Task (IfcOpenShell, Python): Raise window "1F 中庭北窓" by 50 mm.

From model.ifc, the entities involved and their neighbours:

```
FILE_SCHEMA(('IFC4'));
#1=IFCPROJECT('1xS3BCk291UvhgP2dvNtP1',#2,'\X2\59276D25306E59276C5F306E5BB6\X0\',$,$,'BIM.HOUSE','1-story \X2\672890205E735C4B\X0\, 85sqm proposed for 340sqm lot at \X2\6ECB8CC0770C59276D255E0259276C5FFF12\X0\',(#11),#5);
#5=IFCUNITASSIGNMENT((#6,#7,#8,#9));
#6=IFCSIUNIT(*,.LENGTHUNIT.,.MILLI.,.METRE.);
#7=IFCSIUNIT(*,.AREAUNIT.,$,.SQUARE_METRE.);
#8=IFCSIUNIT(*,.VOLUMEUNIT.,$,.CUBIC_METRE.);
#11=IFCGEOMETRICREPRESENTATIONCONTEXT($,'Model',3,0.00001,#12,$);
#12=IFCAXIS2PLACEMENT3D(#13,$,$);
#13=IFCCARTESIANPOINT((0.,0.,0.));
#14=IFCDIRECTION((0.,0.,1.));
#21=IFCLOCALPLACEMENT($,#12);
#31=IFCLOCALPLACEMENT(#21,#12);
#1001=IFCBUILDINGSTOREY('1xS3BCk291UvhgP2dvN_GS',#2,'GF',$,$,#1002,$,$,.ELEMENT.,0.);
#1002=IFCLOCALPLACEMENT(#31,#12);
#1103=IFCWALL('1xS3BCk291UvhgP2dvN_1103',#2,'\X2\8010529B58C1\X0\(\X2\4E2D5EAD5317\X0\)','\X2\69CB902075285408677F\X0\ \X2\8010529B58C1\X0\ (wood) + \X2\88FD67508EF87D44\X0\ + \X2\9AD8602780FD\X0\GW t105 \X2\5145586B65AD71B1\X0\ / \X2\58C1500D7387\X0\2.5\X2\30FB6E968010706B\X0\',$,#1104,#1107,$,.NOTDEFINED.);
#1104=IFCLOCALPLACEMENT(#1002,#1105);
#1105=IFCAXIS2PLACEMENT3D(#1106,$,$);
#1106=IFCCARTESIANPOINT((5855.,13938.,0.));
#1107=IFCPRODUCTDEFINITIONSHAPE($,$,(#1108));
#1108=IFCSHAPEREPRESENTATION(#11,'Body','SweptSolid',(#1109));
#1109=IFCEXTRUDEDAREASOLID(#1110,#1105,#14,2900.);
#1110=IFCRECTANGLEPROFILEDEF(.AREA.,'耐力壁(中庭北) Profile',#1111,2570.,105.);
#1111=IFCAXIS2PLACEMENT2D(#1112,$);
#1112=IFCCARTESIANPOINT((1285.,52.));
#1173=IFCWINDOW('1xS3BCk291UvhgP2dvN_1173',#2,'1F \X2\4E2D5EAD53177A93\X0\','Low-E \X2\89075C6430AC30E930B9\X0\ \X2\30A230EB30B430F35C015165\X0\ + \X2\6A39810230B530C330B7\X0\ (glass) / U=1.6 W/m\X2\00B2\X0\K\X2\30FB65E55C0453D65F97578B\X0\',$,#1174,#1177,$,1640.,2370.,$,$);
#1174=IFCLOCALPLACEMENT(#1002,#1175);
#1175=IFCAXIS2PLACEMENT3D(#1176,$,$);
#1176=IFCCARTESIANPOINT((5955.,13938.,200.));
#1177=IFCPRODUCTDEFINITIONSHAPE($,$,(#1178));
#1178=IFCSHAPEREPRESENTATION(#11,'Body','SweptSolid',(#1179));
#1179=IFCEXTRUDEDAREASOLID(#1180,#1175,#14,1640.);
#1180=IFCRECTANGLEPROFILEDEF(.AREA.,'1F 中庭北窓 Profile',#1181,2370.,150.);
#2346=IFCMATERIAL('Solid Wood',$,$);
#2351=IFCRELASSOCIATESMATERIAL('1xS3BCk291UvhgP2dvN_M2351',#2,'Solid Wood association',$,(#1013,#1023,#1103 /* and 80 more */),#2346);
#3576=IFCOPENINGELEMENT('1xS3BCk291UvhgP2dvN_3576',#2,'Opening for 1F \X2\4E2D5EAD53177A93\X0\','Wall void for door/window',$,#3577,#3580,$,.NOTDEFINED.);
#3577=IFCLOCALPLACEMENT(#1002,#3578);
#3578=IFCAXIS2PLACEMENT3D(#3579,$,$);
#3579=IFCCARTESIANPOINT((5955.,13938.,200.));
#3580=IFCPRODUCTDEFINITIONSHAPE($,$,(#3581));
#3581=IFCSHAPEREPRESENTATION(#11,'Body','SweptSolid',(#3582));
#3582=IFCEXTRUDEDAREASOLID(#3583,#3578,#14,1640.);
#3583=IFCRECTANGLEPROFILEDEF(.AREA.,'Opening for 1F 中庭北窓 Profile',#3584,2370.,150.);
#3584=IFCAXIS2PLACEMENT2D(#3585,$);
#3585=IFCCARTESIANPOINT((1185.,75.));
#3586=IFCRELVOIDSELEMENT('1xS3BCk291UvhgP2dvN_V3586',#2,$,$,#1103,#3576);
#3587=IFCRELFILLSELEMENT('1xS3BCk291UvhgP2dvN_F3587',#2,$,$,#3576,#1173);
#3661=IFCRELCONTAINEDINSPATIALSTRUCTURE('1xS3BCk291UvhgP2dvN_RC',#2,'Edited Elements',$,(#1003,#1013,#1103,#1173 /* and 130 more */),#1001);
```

```python
import numpy as np
import ifcopenshell
import ifcopenshell.api.geometry
import ifcopenshell.util.placement
import ifcopenshell.util.unit

model = ifcopenshell.open("model.ifc")
unit_scale = ifcopenshell.util.unit.calculate_unit_scale(model)

window = model.by_guid("1xS3BCk291UvhgP2dvN_1173")
opening = window.FillsVoids[0].RelatingOpeningElement
dz = 50.0

shift = np.array([0.0, 0.0, dz])
# The window is not placed relative to its opening, so move both.
for product in (opening, window):
    matrix = ifcopenshell.util.placement.get_local_placement(product.ObjectPlacement)
    matrix[:3, 3] += shift
    ifcopenshell.api.geometry.edit_object_placement(model, product=product, matrix=matrix, is_si=False)

print(f"moved by {dz * unit_scale:+.3f} m")

model.write("model_edited.ifc")
```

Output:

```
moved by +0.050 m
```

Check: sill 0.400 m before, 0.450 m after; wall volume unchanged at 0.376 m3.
